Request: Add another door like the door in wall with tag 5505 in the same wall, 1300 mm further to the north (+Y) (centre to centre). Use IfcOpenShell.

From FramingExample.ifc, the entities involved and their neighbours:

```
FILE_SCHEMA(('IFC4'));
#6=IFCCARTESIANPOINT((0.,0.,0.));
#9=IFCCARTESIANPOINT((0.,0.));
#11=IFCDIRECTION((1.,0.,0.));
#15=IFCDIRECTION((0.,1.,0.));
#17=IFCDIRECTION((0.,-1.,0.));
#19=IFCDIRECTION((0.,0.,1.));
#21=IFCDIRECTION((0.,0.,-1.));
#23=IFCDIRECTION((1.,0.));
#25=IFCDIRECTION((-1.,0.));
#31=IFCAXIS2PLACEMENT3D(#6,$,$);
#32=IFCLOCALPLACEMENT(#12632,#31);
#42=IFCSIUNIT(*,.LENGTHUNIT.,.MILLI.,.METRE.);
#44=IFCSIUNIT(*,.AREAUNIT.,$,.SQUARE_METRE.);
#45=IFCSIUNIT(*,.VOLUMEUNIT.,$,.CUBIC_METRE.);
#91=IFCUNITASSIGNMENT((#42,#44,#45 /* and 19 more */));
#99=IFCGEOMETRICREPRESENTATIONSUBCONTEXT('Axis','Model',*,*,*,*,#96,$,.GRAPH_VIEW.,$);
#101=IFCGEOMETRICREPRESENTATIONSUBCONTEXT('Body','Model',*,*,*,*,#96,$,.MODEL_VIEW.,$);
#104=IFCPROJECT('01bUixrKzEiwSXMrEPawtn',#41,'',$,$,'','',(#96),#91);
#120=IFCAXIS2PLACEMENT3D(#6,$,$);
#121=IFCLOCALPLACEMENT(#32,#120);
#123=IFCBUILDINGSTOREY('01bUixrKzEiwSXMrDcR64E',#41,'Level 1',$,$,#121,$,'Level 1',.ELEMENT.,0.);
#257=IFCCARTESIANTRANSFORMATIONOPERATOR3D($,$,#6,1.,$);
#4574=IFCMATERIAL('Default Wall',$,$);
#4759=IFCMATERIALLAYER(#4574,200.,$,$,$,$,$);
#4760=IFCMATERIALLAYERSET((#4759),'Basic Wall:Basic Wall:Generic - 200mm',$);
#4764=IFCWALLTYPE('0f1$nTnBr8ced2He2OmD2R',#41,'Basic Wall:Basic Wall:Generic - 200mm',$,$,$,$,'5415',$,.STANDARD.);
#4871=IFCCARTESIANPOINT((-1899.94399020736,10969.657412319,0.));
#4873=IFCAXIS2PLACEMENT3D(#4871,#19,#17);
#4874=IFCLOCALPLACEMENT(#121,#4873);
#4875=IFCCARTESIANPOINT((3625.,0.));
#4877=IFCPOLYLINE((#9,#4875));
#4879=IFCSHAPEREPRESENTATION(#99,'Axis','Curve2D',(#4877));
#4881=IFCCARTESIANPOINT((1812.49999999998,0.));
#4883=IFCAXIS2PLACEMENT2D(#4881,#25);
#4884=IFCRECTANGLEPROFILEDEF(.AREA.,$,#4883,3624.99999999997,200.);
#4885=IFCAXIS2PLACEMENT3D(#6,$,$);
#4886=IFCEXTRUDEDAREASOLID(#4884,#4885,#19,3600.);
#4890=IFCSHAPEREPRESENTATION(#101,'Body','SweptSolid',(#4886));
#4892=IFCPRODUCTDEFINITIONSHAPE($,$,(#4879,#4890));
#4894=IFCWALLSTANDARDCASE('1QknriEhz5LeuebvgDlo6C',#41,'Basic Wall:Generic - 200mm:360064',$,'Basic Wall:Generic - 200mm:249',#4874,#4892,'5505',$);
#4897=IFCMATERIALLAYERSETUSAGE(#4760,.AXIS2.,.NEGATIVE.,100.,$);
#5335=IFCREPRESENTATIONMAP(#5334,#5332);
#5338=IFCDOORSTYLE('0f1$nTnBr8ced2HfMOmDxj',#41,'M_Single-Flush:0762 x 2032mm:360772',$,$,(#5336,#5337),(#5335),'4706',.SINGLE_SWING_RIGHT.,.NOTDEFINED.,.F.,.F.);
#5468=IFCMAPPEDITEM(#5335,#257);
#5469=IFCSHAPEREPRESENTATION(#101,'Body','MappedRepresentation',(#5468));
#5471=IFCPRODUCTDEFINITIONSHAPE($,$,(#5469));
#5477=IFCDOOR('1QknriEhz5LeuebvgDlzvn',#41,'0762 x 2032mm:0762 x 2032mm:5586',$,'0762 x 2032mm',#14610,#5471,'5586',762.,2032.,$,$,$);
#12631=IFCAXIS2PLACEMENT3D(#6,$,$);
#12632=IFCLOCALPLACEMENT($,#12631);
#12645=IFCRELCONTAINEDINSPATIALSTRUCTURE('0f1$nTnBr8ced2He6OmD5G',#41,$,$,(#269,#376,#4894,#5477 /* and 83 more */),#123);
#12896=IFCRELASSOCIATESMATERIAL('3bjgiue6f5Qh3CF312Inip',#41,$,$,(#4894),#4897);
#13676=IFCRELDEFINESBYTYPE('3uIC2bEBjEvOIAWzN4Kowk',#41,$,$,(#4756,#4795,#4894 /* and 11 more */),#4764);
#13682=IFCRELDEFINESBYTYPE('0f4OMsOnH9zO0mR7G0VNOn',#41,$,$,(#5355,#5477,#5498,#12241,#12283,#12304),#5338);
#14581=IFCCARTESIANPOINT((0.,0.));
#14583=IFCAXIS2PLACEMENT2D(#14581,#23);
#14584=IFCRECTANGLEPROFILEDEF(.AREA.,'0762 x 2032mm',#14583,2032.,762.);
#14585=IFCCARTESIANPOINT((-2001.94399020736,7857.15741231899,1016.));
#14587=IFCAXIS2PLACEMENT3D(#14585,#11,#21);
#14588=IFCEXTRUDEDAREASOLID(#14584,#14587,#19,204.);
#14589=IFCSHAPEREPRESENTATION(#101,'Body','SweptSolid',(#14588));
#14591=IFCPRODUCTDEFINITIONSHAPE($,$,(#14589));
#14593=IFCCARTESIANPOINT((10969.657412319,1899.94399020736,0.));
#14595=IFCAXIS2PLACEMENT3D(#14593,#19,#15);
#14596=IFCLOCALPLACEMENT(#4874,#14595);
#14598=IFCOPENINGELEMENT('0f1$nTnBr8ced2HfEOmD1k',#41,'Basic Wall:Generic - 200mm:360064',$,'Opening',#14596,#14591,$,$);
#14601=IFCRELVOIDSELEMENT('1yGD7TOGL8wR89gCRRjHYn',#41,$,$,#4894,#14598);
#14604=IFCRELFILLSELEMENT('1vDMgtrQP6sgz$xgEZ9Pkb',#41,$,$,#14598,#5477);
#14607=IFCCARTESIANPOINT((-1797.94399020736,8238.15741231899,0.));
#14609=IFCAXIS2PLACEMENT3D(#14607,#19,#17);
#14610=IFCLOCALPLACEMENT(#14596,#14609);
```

```python
import ifcopenshell
import ifcopenshell.api.feature
import ifcopenshell.api.geometry
import ifcopenshell.api.root
import ifcopenshell.geom
import ifcopenshell.util.element
import ifcopenshell.util.placement
import ifcopenshell.util.shape

model = ifcopenshell.open("FramingExample.ifc")
settings = ifcopenshell.geom.settings()


def volume(element):
    """Net volume in cubic metres, openings subtracted."""
    shape = ifcopenshell.geom.create_shape(settings, element)
    return ifcopenshell.util.shape.get_volume(shape.geometry)


def reuse_history(source, copy):
    """copy_class also copies each property set's owner history, people and application; keep the originals."""
    for rel in copy.IsDefinedBy:
        if rel.is_a("IfcRelDefinesByProperties") and (history := rel.RelatingPropertyDefinition.OwnerHistory):
            rel.RelatingPropertyDefinition.OwnerHistory = source.OwnerHistory
            ifcopenshell.util.element.remove_deep2(model, history)


door = model.by_guid("1QknriEhz5LeuebvgDlzvn")
opening = door.FillsVoids[0].RelatingOpeningElement
wall = opening.VoidsElements[0].RelatingBuildingElement
before = volume(wall)
shift = ifcopenshell.util.placement.get_local_placement(wall.ObjectPlacement)[:3, 0] * -1300.0

# copy_class copies the void relationship, type, container and properties, but no geometry.
new_opening = ifcopenshell.api.root.copy_class(model, product=opening)
new_opening.Representation = ifcopenshell.util.element.copy_deep(
    model, opening.Representation, exclude=["IfcGeometricRepresentationContext", "IfcRepresentationMap"]
)
new_opening.Name = "Basic Wall:Generic - 200mm"
new_door = ifcopenshell.api.root.copy_class(model, product=door)
new_door.Representation = ifcopenshell.util.element.copy_deep(
    model, door.Representation, exclude=["IfcGeometricRepresentationContext", "IfcRepresentationMap"]
)
new_door.Name = "0762 x 2032mm:0762 x 2032mm"
new_door.Tag = None
reuse_history(door, new_door)
ifcopenshell.api.feature.add_filling(model, opening=new_opening, element=new_door)

for old, new in ((opening, new_opening), (door, new_door)):
    matrix = ifcopenshell.util.placement.get_local_placement(old.ObjectPlacement)
    matrix[:3, 3] += shift
    ifcopenshell.api.geometry.edit_object_placement(model, product=new, matrix=matrix, is_si=False)

after = volume(wall)

print(f"wall volume {before:.3f} -> {after:.3f} m3")

model.write("FramingExample_rev.ifc")
```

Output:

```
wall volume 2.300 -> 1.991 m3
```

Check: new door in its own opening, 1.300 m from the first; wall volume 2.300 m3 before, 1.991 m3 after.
